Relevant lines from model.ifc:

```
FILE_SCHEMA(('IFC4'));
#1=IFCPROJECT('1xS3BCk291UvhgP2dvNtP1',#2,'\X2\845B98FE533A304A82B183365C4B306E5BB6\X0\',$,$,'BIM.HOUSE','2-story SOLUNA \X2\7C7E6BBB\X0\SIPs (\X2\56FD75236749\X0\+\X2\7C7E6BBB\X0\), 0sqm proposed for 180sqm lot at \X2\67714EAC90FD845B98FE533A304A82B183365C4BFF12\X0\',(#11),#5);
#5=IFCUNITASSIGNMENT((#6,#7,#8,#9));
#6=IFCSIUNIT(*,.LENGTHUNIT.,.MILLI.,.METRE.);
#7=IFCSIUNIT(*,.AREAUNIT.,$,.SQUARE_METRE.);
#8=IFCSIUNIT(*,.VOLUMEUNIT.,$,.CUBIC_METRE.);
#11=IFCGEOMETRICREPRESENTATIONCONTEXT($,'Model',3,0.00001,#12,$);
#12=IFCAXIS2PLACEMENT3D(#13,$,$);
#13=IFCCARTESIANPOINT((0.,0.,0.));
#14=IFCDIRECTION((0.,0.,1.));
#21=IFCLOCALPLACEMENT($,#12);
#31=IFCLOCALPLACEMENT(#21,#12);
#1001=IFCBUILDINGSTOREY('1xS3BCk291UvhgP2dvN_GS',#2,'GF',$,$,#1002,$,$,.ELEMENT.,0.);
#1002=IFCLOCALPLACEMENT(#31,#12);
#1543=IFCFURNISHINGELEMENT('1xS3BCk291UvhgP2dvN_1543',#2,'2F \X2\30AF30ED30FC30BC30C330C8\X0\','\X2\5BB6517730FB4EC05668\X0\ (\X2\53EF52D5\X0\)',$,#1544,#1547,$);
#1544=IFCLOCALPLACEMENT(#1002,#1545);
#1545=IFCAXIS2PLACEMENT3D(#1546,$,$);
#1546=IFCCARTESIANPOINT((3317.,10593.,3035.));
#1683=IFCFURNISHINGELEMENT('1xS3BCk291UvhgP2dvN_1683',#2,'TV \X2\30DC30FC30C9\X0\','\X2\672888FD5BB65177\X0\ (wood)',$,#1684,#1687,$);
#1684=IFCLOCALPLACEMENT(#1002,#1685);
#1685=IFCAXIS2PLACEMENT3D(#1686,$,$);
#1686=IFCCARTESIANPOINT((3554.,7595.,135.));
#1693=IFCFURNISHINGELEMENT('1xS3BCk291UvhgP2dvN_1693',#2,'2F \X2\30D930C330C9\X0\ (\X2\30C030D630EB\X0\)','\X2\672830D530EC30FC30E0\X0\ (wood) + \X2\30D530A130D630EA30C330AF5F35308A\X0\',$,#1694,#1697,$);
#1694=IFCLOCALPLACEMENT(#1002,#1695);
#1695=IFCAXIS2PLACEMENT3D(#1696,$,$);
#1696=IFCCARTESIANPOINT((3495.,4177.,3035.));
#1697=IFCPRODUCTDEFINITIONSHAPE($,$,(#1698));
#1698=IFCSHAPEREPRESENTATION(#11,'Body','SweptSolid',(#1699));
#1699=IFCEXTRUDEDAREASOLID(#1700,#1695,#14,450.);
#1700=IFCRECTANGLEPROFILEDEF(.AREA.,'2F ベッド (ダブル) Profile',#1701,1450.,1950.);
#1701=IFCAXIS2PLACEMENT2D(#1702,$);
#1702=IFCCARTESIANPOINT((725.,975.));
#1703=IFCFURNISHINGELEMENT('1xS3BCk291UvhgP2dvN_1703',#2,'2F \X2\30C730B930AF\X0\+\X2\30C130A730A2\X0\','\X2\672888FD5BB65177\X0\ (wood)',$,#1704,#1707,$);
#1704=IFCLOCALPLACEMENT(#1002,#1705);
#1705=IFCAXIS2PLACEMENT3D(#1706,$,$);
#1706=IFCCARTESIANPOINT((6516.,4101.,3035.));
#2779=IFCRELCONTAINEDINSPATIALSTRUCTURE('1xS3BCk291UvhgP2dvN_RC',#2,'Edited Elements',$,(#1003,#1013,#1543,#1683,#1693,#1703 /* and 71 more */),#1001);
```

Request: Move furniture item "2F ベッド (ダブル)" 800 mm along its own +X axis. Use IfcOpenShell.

```python
import ifcopenshell
import ifcopenshell.api.geometry
import ifcopenshell.util.placement

model = ifcopenshell.open("model.ifc")

item = model.by_guid("1xS3BCk291UvhgP2dvN_1693")
matrix = ifcopenshell.util.placement.get_local_placement(item.ObjectPlacement)
matrix[:3, 3] += matrix[:3, 0] * 800.0
ifcopenshell.api.geometry.edit_object_placement(model, product=item, matrix=matrix, is_si=False)

print(ifcopenshell.util.placement.get_local_placement(item.ObjectPlacement).round(3) + 0.0)

model.write("model-out.ifc")
```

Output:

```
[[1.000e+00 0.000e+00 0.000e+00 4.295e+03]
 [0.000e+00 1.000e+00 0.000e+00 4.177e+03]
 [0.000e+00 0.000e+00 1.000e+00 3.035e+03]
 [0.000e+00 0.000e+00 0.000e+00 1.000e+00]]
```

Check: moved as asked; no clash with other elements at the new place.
